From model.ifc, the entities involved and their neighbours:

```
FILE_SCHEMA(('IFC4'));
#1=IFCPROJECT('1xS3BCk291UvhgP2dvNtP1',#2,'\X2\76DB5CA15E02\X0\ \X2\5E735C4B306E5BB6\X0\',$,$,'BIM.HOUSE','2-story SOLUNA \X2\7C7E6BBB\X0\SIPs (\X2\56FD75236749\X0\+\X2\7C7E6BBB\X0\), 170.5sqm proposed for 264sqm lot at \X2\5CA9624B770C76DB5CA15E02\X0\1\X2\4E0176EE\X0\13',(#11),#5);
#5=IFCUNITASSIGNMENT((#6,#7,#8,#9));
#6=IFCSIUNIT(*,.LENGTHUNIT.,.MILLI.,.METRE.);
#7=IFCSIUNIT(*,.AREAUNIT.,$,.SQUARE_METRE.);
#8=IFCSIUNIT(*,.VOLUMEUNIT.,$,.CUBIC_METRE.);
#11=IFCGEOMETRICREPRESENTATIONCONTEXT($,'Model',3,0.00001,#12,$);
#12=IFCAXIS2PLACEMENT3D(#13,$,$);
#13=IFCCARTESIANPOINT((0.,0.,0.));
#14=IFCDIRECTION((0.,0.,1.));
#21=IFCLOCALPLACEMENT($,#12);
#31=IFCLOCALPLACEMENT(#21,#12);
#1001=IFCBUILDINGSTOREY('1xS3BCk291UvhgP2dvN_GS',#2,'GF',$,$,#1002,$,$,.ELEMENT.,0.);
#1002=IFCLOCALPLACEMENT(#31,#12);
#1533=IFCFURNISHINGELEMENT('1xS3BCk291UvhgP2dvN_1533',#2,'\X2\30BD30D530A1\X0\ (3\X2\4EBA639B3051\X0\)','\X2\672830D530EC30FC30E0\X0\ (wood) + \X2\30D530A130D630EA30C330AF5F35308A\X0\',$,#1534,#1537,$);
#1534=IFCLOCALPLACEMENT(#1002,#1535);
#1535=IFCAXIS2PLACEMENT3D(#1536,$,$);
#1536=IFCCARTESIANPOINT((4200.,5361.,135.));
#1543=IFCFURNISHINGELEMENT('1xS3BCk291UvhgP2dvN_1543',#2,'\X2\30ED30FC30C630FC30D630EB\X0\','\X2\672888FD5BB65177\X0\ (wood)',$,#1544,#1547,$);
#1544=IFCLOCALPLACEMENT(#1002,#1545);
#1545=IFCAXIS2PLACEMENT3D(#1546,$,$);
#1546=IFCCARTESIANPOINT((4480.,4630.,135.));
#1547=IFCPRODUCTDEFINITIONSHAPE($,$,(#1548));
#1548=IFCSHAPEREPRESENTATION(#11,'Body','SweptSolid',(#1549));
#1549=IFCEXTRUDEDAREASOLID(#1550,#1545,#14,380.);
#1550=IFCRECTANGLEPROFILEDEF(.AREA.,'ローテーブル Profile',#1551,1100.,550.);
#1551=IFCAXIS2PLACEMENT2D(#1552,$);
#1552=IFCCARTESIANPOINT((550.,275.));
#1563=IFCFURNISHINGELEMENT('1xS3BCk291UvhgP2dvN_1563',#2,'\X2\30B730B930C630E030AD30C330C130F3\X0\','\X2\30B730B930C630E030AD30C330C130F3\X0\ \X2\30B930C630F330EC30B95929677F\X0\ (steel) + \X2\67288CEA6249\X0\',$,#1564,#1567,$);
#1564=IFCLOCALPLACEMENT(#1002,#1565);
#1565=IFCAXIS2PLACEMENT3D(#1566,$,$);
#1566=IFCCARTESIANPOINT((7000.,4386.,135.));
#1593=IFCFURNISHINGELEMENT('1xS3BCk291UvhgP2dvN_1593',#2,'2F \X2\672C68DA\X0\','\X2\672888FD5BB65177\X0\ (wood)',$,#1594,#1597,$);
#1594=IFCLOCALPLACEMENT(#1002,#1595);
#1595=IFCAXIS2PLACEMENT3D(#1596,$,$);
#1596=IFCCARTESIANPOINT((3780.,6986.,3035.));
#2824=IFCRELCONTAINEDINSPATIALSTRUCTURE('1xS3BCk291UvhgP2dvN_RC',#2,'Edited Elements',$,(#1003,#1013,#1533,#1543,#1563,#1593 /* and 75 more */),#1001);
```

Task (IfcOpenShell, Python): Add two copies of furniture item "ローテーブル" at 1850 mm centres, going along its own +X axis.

```python
import ifcopenshell
import ifcopenshell.api.geometry
import ifcopenshell.api.root
import ifcopenshell.util.element
import ifcopenshell.util.placement
import ifcopenshell.util.unit

model = ifcopenshell.open("model.ifc")
unit_scale = ifcopenshell.util.unit.calculate_unit_scale(model)


def reuse_history(source, copy):
    """copy_class also copies each property set's owner history, people and application; keep the originals."""
    for rel in copy.IsDefinedBy:
        if rel.is_a("IfcRelDefinesByProperties") and (history := rel.RelatingPropertyDefinition.OwnerHistory):
            rel.RelatingPropertyDefinition.OwnerHistory = source.OwnerHistory
            ifcopenshell.util.element.remove_deep2(model, history)


source = model.by_guid("1xS3BCk291UvhgP2dvN_1543")
base = ifcopenshell.util.placement.get_local_placement(source.ObjectPlacement)
step = base[:3, 0] * 1.85 / unit_scale

for i in range(1, 3):
    copy = ifcopenshell.api.root.copy_class(model, product=source)
    copy.Representation = ifcopenshell.util.element.copy_deep(
        model, source.Representation, exclude=["IfcGeometricRepresentationContext", "IfcRepresentationMap"]
    )
    reuse_history(source, copy)
    matrix = base.copy()
    matrix[:3, 3] += i * step
    print("added at", matrix[:3, 3].round(3) + 0.0)
    ifcopenshell.api.geometry.edit_object_placement(model, product=copy, matrix=matrix, is_si=False)

model.write("model-out.ifc")
```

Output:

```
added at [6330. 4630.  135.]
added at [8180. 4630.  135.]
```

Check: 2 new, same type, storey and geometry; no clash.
